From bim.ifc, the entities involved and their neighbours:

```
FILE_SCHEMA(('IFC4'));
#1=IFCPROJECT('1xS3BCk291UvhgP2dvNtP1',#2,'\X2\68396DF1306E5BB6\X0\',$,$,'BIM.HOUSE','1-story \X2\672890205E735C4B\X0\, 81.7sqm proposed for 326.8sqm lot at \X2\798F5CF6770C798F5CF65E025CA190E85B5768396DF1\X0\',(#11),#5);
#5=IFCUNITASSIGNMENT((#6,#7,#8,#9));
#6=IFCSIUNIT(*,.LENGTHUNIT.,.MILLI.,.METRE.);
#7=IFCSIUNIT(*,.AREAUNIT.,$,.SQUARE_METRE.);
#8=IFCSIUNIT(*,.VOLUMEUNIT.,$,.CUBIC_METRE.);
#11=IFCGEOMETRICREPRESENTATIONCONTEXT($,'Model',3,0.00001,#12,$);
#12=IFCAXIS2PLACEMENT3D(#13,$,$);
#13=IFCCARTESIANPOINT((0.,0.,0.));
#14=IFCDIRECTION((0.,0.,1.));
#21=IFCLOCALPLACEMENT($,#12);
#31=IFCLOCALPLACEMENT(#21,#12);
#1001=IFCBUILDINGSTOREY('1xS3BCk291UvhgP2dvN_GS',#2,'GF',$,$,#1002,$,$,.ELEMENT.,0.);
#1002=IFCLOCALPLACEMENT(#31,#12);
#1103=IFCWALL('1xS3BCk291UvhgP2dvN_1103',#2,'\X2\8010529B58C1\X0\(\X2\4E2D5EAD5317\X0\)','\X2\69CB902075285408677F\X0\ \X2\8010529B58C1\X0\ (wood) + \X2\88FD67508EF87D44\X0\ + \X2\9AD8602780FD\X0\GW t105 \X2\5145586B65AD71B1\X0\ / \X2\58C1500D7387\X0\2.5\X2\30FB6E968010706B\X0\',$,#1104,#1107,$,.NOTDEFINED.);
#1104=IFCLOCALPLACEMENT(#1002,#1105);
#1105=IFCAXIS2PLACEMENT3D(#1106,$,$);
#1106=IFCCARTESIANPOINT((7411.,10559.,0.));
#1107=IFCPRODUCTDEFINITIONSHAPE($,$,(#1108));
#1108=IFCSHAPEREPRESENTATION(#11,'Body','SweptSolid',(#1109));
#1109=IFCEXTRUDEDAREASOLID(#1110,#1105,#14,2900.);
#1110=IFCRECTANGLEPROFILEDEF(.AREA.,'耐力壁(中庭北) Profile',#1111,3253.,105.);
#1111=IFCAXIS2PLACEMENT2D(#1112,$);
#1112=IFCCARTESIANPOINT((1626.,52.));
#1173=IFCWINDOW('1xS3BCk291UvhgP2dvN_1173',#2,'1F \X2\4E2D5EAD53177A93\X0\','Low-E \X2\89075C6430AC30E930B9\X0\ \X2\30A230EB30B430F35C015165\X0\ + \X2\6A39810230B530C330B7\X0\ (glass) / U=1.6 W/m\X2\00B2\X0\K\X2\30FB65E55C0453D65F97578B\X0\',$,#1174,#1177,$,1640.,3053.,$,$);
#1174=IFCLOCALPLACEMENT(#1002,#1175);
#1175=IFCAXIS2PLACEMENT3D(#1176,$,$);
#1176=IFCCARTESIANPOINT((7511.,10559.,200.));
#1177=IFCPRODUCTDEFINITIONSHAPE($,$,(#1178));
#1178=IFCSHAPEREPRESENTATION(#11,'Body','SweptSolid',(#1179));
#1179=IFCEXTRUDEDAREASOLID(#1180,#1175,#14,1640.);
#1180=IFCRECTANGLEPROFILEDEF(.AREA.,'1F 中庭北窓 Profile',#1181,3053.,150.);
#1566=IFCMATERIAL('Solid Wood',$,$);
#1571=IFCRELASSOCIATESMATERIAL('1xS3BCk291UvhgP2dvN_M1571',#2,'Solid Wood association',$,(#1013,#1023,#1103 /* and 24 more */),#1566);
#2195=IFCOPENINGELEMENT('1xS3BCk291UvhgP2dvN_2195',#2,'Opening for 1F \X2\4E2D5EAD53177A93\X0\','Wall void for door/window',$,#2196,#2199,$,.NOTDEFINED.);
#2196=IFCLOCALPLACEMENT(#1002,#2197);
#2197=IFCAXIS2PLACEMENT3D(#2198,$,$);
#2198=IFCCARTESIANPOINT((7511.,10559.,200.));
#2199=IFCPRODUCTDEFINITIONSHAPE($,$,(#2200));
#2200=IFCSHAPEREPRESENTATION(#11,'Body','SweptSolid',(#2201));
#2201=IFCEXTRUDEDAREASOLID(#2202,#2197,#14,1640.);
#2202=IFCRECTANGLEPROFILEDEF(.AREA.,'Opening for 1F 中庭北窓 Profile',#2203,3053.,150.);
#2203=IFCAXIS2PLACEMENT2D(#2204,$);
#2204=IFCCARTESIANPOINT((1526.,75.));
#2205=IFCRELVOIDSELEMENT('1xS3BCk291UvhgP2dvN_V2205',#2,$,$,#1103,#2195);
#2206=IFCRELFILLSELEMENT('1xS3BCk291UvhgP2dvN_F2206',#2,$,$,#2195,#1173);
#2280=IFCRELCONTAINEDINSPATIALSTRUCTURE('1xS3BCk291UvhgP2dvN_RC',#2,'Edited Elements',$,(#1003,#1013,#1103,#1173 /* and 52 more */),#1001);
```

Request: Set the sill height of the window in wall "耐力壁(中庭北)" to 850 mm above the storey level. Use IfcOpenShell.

```python
import numpy as np
import ifcopenshell
import ifcopenshell.api.geometry
import ifcopenshell.geom
import ifcopenshell.util.element
import ifcopenshell.util.placement
import ifcopenshell.util.shape
import ifcopenshell.util.unit

model = ifcopenshell.open("bim.ifc")
unit_scale = ifcopenshell.util.unit.calculate_unit_scale(model)

window = model.by_guid("1xS3BCk291UvhgP2dvN_1173")
opening = window.FillsVoids[0].RelatingOpeningElement
storey = ifcopenshell.util.element.get_container(window, ifc_class="IfcBuildingStorey")
level = ifcopenshell.util.placement.get_local_placement(storey.ObjectPlacement)[2, 3]

# The opening's origin need not be at the sill, so measure its lowest point.
shape = ifcopenshell.geom.create_shape(ifcopenshell.geom.settings(), opening)
bottom = ifcopenshell.util.shape.get_shape_bottom_elevation(shape, shape.geometry) / unit_scale
dz = level + 850.0 - bottom

shift = np.array([0.0, 0.0, dz])
# The window is not placed relative to its opening, so move both.
for product in (opening, window):
    matrix = ifcopenshell.util.placement.get_local_placement(product.ObjectPlacement)
    matrix[:3, 3] += shift
    ifcopenshell.api.geometry.edit_object_placement(model, product=product, matrix=matrix, is_si=False)

print(f"moved by {dz * unit_scale:+.3f} m")

model.write("bim_rev.ifc")
```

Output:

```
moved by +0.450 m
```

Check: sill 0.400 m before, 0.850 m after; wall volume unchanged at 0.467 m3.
